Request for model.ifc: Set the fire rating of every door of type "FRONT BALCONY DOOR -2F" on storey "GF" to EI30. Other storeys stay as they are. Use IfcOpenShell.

First a look at what the model holds.

```python
import ifcopenshell
import ifcopenshell.util.element

model = ifcopenshell.open("model.ifc")
print(model.schema)
storey = next(s for s in model.by_type("IfcBuildingStorey") if s.Name == "GF")
doors = [e for e in ifcopenshell.util.element.get_decomposition(storey) if e.is_a("IfcDoor")]
seen = {}
for e in doors:
    element_type = ifcopenshell.util.element.get_type(e)
    key = (element_type.Name if element_type != e and element_type else None, ifcopenshell.util.element.get_pset(e, "Pset_DoorCommon", "FireRating"))
    seen[key] = seen.get(key, 0) + 1
for (name, value), count in sorted(seen.items(), key=str):
    print(count, "x", name, "|", value)
```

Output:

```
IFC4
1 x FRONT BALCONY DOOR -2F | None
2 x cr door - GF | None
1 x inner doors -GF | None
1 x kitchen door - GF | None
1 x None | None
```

```python
import ifcopenshell
import ifcopenshell.api.pset
import ifcopenshell.util.element

model = ifcopenshell.open("model.ifc")

storey = next(s for s in model.by_type("IfcBuildingStorey") if s.Name == "GF")
doors = [e for e in ifcopenshell.util.element.get_decomposition(storey) if e.is_a("IfcDoor")]

count = 0
for e in doors:
    element_type = ifcopenshell.util.element.get_type(e)
    if element_type in (None, e) or element_type.Name != "FRONT BALCONY DOOR -2F":
        continue
    # add_pset returns the element's existing set when there is one.
    pset = ifcopenshell.api.pset.add_pset(model, product=e, name="Pset_DoorCommon")
    ifcopenshell.api.pset.edit_pset(model, pset=pset, properties={"FireRating": "EI30"})
    count += 1

print(count, "doors updated")

model.write("model-out.ifc")
```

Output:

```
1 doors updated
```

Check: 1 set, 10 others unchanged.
